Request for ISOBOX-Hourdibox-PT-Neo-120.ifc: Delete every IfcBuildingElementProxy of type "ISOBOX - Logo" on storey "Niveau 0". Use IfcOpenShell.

First a look at what the model holds.

```python
import ifcopenshell
import ifcopenshell.util.element

model = ifcopenshell.open("ISOBOX-Hourdibox-PT-Neo-120.ifc")
print(model.schema)
storey = next(s for s in model.by_type("IfcBuildingStorey") if s.Name == "Niveau 0")
proxies = [e for e in ifcopenshell.util.element.get_decomposition(storey) if e.is_a("IfcBuildingElementProxy")]
seen = {}
for e in proxies:
    element_type = ifcopenshell.util.element.get_type(e)
    name = element_type.Name if element_type not in (None, e) else None
    seen[name] = seen.get(name, 0) + 1
for name, count in sorted(seen.items(), key=str):
    print(count, "x", name)
```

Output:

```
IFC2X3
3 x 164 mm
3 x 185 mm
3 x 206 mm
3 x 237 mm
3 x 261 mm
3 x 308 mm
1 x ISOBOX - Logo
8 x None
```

```python
import ifcopenshell
import ifcopenshell.api.root
import ifcopenshell.util.element

model = ifcopenshell.open("ISOBOX-Hourdibox-PT-Neo-120.ifc")

storey = next(s for s in model.by_type("IfcBuildingStorey") if s.Name == "Niveau 0")
proxies = [e for e in ifcopenshell.util.element.get_decomposition(storey) if e.is_a("IfcBuildingElementProxy")]
targets = [e for e in proxies if (t := ifcopenshell.util.element.get_type(e)) not in (None, e) and t.Name == "ISOBOX - Logo"]

for e in targets:
    ifcopenshell.api.root.remove_product(model, product=e)
print(len(targets), "removed")

model.write("ISOBOX-Hourdibox-PT-Neo-120-out.ifc")
```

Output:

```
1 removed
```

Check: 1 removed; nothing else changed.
